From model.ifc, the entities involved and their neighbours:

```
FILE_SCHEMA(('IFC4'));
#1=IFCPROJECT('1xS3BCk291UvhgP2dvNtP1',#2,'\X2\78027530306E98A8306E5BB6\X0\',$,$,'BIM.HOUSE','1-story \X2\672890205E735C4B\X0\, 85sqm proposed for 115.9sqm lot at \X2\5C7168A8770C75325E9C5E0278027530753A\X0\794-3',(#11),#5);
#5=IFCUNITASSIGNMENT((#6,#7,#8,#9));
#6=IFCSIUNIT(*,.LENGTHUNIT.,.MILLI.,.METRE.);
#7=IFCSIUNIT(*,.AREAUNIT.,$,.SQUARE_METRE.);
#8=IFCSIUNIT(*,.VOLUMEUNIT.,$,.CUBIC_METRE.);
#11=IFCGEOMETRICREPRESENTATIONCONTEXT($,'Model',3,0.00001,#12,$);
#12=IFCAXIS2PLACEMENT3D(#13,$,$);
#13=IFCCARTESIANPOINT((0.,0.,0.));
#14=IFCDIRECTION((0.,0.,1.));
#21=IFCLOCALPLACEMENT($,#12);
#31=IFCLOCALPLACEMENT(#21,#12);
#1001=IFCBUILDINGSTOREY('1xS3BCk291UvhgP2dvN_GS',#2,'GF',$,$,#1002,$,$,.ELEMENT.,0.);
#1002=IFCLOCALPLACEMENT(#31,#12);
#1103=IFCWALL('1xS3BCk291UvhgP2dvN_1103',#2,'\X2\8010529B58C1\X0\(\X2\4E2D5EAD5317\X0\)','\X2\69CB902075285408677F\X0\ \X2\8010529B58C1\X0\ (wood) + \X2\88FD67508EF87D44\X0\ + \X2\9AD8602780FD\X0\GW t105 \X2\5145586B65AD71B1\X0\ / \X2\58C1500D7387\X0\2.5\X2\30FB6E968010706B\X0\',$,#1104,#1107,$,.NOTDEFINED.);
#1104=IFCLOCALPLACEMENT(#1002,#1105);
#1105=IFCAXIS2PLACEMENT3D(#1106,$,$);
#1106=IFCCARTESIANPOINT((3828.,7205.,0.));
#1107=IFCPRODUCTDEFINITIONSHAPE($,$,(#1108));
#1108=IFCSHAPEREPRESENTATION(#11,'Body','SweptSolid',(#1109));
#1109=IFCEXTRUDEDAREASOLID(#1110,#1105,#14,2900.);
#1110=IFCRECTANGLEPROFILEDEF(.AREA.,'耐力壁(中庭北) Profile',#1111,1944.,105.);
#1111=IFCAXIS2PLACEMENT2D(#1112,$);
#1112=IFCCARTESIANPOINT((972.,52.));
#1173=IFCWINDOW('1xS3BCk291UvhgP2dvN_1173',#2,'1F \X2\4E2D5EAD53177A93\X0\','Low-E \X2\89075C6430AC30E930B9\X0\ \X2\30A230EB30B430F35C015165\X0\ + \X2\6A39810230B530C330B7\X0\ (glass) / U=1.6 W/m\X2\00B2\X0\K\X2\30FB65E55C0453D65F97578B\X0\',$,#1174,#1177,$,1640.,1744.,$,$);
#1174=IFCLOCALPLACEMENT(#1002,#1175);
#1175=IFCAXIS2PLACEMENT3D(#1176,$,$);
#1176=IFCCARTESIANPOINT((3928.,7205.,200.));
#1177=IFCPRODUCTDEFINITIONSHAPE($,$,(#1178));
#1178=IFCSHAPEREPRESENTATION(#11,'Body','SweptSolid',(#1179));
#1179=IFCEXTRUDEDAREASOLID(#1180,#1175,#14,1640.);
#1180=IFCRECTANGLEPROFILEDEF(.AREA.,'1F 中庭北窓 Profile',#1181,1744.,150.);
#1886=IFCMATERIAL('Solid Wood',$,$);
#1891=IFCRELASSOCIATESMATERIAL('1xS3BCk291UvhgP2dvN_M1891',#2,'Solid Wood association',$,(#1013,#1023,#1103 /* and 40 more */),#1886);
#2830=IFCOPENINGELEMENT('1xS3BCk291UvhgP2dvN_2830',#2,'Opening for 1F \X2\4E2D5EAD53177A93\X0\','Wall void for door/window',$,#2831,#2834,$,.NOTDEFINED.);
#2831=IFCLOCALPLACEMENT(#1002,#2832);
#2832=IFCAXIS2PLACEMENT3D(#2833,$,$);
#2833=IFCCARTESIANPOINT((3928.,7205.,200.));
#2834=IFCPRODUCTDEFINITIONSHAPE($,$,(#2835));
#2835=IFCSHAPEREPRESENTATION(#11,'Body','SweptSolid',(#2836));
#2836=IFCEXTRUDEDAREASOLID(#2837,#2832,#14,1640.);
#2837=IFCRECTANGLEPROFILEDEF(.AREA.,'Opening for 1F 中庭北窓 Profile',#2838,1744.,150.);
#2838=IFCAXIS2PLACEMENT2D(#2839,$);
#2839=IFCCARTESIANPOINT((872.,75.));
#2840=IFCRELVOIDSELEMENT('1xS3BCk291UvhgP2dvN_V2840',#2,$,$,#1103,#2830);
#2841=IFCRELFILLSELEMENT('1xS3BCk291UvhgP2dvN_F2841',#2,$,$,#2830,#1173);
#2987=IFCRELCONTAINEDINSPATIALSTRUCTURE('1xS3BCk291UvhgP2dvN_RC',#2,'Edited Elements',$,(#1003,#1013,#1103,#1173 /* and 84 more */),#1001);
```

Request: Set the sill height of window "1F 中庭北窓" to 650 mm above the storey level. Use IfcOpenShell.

```python
import numpy as np
import ifcopenshell
import ifcopenshell.api.geometry
import ifcopenshell.geom
import ifcopenshell.util.element
import ifcopenshell.util.placement
import ifcopenshell.util.shape
import ifcopenshell.util.unit

model = ifcopenshell.open("model.ifc")
unit_scale = ifcopenshell.util.unit.calculate_unit_scale(model)

window = model.by_id(1173)
opening = window.FillsVoids[0].RelatingOpeningElement
storey = ifcopenshell.util.element.get_container(window, ifc_class="IfcBuildingStorey")
level = ifcopenshell.util.placement.get_local_placement(storey.ObjectPlacement)[2, 3]

# The opening's origin need not be at the sill, so measure its lowest point.
shape = ifcopenshell.geom.create_shape(ifcopenshell.geom.settings(), opening)
bottom = ifcopenshell.util.shape.get_shape_bottom_elevation(shape, shape.geometry) / unit_scale
dz = level + 0.65 / unit_scale - bottom

shift = np.array([0.0, 0.0, dz])
# The window is not placed relative to its opening, so move both.
for product in (opening, window):
    matrix = ifcopenshell.util.placement.get_local_placement(product.ObjectPlacement)
    matrix[:3, 3] += shift
    ifcopenshell.api.geometry.edit_object_placement(model, product=product, matrix=matrix, is_si=False)

print(f"moved by {dz * unit_scale:+.3f} m")

model.write("model-out.ifc")
```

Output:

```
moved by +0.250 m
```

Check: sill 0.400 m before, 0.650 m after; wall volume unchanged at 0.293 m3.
